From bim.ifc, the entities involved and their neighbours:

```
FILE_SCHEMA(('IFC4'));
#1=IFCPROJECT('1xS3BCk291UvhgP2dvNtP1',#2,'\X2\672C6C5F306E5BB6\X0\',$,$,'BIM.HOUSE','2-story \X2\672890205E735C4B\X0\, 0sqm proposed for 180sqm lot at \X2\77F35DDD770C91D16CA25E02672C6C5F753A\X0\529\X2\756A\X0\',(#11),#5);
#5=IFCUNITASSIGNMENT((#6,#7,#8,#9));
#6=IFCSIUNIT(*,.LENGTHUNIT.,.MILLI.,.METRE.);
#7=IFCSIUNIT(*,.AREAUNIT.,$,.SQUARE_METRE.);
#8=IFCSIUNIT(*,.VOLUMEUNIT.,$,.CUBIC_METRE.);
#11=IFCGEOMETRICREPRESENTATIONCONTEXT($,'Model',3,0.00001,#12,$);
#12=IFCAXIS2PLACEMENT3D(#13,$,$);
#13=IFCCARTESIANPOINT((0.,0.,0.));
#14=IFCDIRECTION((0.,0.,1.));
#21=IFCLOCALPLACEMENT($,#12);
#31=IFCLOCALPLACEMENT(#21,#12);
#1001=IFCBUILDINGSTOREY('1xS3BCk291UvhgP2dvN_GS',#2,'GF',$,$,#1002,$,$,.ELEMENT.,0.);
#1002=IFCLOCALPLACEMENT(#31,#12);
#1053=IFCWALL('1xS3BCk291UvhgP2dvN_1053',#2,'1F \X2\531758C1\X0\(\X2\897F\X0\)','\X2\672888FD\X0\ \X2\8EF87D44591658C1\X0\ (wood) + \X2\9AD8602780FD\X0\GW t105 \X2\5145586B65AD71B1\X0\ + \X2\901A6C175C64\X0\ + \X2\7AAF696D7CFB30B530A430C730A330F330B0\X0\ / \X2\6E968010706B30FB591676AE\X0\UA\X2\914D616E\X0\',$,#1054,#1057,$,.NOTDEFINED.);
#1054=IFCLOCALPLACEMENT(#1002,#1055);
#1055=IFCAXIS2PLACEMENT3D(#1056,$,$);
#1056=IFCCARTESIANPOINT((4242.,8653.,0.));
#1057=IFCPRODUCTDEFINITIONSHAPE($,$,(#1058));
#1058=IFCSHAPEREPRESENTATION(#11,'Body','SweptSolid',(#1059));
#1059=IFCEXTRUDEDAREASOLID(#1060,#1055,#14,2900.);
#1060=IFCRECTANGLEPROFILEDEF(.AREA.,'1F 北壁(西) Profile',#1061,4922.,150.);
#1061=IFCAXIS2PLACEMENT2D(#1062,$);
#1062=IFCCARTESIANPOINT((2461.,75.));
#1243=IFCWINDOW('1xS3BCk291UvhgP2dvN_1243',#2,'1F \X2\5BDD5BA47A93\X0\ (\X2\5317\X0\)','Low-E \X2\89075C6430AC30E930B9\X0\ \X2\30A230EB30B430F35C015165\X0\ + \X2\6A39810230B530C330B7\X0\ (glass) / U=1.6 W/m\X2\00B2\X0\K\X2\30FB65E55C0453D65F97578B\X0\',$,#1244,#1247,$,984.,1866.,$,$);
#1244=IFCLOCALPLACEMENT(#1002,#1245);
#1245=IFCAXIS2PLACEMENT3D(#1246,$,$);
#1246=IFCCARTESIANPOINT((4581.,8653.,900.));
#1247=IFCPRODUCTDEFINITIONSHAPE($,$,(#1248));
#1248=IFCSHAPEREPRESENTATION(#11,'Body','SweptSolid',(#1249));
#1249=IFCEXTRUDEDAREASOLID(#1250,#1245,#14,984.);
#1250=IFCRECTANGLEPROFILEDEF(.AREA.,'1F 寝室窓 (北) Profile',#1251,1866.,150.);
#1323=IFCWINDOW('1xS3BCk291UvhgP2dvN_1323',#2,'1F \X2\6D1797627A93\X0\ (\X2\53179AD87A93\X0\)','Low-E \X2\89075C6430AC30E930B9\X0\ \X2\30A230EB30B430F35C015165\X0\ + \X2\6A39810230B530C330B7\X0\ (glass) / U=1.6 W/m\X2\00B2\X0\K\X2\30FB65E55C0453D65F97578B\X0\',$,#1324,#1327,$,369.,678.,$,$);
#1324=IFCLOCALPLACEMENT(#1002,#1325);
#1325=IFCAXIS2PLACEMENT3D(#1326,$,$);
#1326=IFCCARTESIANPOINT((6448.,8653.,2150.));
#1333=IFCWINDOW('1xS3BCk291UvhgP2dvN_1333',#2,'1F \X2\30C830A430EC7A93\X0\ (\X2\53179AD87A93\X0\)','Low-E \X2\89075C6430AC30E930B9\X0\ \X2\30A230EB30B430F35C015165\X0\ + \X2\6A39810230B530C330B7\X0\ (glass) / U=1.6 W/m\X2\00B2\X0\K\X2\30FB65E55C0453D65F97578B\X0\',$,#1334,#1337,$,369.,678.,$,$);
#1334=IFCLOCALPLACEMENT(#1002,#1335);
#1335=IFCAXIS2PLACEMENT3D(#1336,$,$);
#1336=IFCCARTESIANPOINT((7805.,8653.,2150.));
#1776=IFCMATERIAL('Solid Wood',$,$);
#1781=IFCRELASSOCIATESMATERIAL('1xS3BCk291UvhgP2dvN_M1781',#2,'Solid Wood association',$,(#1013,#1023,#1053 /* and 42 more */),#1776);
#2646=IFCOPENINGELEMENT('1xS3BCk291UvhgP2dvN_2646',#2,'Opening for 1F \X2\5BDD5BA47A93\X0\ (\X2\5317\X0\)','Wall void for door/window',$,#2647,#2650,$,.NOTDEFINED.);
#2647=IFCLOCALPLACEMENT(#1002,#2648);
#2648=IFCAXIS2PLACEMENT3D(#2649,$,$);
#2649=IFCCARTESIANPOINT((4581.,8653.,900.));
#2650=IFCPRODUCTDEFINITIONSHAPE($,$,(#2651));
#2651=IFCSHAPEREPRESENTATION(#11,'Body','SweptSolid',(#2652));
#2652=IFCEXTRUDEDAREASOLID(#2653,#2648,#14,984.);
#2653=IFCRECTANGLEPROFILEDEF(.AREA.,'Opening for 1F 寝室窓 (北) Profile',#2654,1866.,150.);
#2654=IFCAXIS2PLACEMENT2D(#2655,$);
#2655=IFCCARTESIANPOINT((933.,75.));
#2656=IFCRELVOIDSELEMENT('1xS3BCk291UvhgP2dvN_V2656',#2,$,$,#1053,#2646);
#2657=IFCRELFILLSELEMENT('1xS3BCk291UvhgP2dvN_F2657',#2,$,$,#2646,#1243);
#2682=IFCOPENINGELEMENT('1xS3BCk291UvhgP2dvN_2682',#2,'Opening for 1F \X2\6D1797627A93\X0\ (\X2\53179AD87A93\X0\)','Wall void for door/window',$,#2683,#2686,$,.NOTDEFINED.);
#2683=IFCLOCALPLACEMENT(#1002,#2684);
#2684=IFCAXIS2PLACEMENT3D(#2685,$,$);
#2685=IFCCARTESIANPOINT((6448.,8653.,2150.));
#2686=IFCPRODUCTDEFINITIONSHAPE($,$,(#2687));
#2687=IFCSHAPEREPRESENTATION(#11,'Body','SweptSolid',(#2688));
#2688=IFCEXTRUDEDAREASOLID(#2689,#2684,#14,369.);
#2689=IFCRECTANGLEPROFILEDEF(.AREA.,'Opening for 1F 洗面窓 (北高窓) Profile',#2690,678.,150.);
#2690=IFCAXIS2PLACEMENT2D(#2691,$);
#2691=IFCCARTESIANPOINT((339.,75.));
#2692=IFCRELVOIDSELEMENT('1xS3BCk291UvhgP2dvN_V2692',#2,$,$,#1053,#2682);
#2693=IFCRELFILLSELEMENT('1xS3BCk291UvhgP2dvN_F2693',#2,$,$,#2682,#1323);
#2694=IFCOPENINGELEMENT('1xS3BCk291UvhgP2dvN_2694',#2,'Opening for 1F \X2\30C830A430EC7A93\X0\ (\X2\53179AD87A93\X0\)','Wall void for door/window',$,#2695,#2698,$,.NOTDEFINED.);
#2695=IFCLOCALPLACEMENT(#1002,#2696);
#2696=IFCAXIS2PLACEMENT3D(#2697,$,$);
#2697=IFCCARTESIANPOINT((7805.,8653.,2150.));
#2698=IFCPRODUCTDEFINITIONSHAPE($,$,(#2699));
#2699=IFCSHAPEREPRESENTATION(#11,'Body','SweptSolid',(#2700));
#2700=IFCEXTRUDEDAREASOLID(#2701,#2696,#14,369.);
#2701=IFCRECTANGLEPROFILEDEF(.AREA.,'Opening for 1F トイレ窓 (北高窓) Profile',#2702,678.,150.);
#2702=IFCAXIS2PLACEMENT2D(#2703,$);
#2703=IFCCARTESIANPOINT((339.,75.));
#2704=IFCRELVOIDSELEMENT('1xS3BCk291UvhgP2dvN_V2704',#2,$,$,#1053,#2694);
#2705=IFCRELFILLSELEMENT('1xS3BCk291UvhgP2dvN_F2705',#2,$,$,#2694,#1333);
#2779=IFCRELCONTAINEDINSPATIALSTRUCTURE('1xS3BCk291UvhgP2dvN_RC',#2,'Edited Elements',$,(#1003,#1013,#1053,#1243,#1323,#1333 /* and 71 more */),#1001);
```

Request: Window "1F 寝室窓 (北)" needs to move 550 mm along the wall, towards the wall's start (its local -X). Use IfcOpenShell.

```python
import ifcopenshell
import ifcopenshell.api.geometry
import ifcopenshell.util.placement
import ifcopenshell.util.unit

model = ifcopenshell.open("bim.ifc")
unit_scale = ifcopenshell.util.unit.calculate_unit_scale(model)

window = model.by_id(1243)
opening = window.FillsVoids[0].RelatingOpeningElement
wall = opening.VoidsElements[0].RelatingBuildingElement

wall_matrix = ifcopenshell.util.placement.get_local_placement(wall.ObjectPlacement)
shift = wall_matrix[:3, 0] * -0.55 / unit_scale
before = ifcopenshell.util.placement.get_local_placement(window.ObjectPlacement)[:3, 3].copy()

# The window is not placed relative to its opening, so move both.
for product in (opening, window):
    matrix = ifcopenshell.util.placement.get_local_placement(product.ObjectPlacement)
    matrix[:3, 3] += shift
    ifcopenshell.api.geometry.edit_object_placement(model, product=product, matrix=matrix, is_si=False)

after = ifcopenshell.util.placement.get_local_placement(window.ObjectPlacement)[:3, 3]
print("window moved by", (after - before).round(3) + 0.0)

model.write("bim_v2.ifc")
```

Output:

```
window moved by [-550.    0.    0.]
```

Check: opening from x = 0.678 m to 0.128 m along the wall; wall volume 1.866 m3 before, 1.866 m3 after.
